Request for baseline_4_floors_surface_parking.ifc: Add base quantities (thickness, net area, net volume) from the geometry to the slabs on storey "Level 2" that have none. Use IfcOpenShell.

First a look at what the model holds.

```python
import ifcopenshell
import ifcopenshell.util.element
import ifcopenshell.util.unit

model = ifcopenshell.open("baseline_4_floors_surface_parking.ifc")
print(model.schema)
for unit_type in ("LENGTHUNIT", "AREAUNIT", "VOLUMEUNIT"):
    print(unit_type, ifcopenshell.util.unit.calculate_unit_scale(model, unit_type))
storey = next(s for s in model.by_type("IfcBuildingStorey") if s.Name == "Level 2")
slabs = [e for e in ifcopenshell.util.element.get_decomposition(storey) if e.is_a("IfcSlab")]
for e in sorted(slabs, key=lambda e: e.id()):
    print(e.id(), e.is_a(), e.Name, list(ifcopenshell.util.element.get_psets(e, qtos_only=True)), sep=" | ")
```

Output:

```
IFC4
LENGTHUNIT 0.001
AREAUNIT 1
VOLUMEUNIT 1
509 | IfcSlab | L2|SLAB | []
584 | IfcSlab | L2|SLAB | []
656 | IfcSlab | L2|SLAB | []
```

```python
import ifcopenshell
import ifcopenshell.api.pset
import ifcopenshell.geom
import ifcopenshell.util.element
import ifcopenshell.util.shape
import ifcopenshell.util.unit

model = ifcopenshell.open("baseline_4_floors_surface_parking.ifc")
unit_scale = ifcopenshell.util.unit.calculate_unit_scale(model)
area_scale = ifcopenshell.util.unit.calculate_unit_scale(model, "AREAUNIT")
volume_scale = ifcopenshell.util.unit.calculate_unit_scale(model, "VOLUMEUNIT")
settings = ifcopenshell.geom.settings()

storey = next(s for s in model.by_type("IfcBuildingStorey") if s.Name == "Level 2")
slabs = [e for e in ifcopenshell.util.element.get_decomposition(storey) if e.is_a("IfcSlab")]

for e in sorted(slabs, key=lambda e: e.id()):
    if ifcopenshell.util.element.get_psets(e, qtos_only=True, should_inherit=False):
        continue
    # Geometry comes back in metres, in the element's own axes.
    shape = ifcopenshell.geom.create_shape(settings, e)
    values = {
        "Width": ifcopenshell.util.shape.get_z(shape.geometry) / unit_scale,
        "NetArea": ifcopenshell.util.shape.get_footprint_area(shape.geometry) / area_scale,
        "NetVolume": ifcopenshell.util.shape.get_volume(shape.geometry) / volume_scale,
    }
    qto = ifcopenshell.api.pset.add_qto(model, product=e, name="Qto_SlabBaseQuantities")
    ifcopenshell.api.pset.edit_qto(model, qto=qto, properties=values)
    print(e.id(), {k: round(v, 3) for k, v in values.items()})

model.write("baseline_4_floors_surface_parking_v2.ifc")
```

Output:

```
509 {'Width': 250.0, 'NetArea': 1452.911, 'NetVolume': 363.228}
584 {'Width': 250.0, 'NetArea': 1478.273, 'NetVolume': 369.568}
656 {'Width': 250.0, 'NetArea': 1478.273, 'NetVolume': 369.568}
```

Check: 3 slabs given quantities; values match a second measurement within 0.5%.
